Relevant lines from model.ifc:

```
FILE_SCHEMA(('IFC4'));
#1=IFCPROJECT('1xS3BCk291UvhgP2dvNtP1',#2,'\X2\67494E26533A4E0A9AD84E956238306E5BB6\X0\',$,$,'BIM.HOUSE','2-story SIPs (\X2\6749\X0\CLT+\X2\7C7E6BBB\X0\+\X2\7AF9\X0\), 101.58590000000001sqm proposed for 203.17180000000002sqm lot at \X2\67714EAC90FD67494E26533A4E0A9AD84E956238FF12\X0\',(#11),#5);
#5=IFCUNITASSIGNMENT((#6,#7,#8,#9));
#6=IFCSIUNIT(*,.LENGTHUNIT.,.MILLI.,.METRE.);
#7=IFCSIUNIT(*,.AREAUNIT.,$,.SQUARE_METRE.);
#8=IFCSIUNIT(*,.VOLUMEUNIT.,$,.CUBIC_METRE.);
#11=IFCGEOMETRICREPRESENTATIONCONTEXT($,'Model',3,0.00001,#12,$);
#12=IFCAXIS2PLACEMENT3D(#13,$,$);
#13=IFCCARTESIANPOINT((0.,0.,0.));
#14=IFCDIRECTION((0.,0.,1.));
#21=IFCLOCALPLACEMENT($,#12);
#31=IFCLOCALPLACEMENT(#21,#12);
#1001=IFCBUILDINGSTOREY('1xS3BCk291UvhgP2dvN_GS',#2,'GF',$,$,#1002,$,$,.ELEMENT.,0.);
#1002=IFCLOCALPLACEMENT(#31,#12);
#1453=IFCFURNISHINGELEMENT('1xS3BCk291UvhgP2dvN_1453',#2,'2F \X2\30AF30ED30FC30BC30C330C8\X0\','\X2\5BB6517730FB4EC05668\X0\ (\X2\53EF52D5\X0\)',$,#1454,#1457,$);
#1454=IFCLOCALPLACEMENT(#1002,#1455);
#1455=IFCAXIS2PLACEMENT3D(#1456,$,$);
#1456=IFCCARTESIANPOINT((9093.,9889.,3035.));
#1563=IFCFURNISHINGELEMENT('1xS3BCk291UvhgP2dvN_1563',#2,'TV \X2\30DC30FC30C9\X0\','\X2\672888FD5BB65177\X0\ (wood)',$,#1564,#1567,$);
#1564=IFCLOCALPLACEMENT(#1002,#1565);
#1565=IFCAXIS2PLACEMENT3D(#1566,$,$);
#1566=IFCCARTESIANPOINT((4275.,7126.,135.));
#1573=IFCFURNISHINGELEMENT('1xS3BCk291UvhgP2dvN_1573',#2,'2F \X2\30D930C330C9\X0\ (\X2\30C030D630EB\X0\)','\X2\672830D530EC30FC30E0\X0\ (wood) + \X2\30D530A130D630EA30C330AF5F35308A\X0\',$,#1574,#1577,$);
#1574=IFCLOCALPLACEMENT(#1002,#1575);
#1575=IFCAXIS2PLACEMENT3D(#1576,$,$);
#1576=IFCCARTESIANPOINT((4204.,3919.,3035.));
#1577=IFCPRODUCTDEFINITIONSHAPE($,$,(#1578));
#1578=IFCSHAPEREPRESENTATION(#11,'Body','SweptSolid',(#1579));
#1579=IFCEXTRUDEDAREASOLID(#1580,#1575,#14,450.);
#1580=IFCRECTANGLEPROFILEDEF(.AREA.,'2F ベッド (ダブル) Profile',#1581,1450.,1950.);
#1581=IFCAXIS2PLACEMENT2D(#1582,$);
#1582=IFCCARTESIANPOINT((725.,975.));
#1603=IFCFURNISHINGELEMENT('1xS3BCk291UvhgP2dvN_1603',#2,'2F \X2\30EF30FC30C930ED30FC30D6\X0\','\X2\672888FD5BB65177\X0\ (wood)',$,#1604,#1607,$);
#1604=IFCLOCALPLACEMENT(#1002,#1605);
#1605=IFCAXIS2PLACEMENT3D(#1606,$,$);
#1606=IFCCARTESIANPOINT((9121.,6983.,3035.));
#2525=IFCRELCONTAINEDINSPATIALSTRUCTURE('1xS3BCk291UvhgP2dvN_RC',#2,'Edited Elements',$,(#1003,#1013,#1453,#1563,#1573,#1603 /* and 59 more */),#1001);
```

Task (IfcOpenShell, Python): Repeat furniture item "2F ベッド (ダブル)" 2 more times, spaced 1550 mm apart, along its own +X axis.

```python
import ifcopenshell
import ifcopenshell.api.geometry
import ifcopenshell.api.root
import ifcopenshell.util.element
import ifcopenshell.util.placement
import ifcopenshell.util.unit

model = ifcopenshell.open("model.ifc")
unit_scale = ifcopenshell.util.unit.calculate_unit_scale(model)


def reuse_history(source, copy):
    """copy_class also copies each property set's owner history, people and application; keep the originals."""
    for rel in copy.IsDefinedBy:
        if rel.is_a("IfcRelDefinesByProperties") and (history := rel.RelatingPropertyDefinition.OwnerHistory):
            rel.RelatingPropertyDefinition.OwnerHistory = source.OwnerHistory
            ifcopenshell.util.element.remove_deep2(model, history)


source = model.by_guid("1xS3BCk291UvhgP2dvN_1573")
base = ifcopenshell.util.placement.get_local_placement(source.ObjectPlacement)
step = base[:3, 0] * 1.55 / unit_scale

for i in range(1, 3):
    copy = ifcopenshell.api.root.copy_class(model, product=source)
    copy.Representation = ifcopenshell.util.element.copy_deep(
        model, source.Representation, exclude=["IfcGeometricRepresentationContext", "IfcRepresentationMap"]
    )
    reuse_history(source, copy)
    matrix = base.copy()
    matrix[:3, 3] += i * step
    print("added at", matrix[:3, 3].round(3) + 0.0)
    ifcopenshell.api.geometry.edit_object_placement(model, product=copy, matrix=matrix, is_si=False)

model.write("model_updated.ifc")
```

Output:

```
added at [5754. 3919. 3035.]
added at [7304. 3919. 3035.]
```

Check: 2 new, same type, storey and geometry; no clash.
